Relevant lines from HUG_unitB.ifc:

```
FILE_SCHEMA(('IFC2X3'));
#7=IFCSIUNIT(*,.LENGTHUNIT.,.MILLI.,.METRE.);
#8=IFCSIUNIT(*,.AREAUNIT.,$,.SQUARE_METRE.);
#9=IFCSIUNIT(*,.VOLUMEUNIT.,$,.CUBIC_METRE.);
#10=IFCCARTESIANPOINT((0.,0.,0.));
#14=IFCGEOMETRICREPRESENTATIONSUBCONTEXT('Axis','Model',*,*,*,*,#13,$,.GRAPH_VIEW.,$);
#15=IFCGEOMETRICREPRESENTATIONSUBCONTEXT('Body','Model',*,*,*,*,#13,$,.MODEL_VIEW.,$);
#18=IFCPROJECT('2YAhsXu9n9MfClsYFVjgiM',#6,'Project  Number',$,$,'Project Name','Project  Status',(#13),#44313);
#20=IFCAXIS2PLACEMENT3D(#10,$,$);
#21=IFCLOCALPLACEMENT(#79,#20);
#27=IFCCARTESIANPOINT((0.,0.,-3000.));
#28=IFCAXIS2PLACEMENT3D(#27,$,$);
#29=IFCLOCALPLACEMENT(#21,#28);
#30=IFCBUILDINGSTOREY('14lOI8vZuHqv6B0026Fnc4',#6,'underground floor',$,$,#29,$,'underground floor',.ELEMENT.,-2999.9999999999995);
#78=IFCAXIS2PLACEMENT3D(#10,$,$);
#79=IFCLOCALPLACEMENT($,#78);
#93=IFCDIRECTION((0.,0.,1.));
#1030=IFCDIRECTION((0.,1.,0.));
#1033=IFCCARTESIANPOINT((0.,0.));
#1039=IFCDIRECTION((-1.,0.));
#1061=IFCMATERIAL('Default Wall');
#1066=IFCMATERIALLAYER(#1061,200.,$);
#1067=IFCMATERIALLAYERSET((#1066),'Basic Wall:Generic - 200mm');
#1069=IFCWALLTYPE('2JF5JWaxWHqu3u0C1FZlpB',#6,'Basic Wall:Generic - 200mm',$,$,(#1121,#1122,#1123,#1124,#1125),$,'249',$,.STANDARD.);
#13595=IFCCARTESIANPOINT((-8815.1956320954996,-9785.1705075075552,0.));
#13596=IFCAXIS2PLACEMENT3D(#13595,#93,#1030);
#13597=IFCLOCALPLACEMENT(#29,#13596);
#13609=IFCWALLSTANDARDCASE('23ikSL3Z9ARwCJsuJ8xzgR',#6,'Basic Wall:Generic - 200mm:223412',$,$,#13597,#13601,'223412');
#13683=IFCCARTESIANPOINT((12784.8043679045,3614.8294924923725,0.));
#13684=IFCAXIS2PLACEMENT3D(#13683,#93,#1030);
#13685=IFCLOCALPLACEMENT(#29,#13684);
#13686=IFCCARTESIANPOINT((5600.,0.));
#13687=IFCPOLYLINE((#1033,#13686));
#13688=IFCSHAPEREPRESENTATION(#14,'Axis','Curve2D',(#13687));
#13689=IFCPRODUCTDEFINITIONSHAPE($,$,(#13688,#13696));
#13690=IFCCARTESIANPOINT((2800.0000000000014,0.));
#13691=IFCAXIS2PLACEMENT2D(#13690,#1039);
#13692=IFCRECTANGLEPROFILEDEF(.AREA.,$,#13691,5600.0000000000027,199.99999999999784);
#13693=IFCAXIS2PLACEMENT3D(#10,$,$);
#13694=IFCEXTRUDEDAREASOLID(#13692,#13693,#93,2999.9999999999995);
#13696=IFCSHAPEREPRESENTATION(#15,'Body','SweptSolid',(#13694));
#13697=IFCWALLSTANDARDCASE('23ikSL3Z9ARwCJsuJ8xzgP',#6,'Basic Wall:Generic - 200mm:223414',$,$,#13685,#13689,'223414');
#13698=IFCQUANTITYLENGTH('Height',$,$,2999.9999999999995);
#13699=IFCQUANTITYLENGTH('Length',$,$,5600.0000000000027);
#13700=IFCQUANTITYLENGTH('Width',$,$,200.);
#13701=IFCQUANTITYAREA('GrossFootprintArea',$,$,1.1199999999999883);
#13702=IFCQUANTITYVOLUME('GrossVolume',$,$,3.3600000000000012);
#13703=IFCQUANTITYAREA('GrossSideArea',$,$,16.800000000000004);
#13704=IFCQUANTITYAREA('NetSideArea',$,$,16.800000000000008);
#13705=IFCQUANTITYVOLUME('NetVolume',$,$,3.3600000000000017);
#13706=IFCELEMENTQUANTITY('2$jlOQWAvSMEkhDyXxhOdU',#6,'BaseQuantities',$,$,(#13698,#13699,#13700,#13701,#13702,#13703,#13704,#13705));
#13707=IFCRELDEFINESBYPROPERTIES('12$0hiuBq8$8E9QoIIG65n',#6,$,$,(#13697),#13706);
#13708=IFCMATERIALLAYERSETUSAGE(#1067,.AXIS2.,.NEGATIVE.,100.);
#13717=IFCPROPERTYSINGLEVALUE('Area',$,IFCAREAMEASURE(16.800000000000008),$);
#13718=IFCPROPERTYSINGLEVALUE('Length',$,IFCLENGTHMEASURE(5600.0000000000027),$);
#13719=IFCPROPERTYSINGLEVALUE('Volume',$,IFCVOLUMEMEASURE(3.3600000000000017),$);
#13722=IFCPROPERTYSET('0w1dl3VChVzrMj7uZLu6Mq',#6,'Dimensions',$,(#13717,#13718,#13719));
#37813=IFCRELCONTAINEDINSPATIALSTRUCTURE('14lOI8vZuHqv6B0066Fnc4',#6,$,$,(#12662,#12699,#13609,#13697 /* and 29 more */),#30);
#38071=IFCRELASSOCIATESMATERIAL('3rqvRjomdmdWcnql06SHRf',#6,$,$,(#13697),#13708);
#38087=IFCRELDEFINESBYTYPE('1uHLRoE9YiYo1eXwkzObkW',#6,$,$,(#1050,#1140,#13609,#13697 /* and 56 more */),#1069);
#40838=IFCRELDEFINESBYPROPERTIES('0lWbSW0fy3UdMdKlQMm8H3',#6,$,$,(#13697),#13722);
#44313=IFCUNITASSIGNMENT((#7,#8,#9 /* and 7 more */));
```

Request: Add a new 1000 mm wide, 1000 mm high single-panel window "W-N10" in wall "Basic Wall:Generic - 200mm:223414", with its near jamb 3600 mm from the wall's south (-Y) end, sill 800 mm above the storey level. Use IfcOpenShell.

```python
import numpy as np
import ifcopenshell
import ifcopenshell.api.feature
import ifcopenshell.api.geometry
import ifcopenshell.api.pset
import ifcopenshell.api.root
import ifcopenshell.api.spatial
import ifcopenshell.api.type
import ifcopenshell.geom
import ifcopenshell.util.element
import ifcopenshell.util.placement
import ifcopenshell.util.representation
import ifcopenshell.util.shape
import ifcopenshell.util.unit

model = ifcopenshell.open("HUG_unitB.ifc")
unit_scale = ifcopenshell.util.unit.calculate_unit_scale(model)
area_scale = ifcopenshell.util.unit.calculate_unit_scale(model, "AREAUNIT")
volume_scale = ifcopenshell.util.unit.calculate_unit_scale(model, "VOLUMEUNIT")
settings = ifcopenshell.geom.settings()


def volume(element):
    """Net volume in cubic metres, openings subtracted."""
    shape = ifcopenshell.geom.create_shape(settings, element)
    return ifcopenshell.util.shape.get_volume(shape.geometry)


wall = model.by_guid("23ikSL3Z9ARwCJsuJ8xzgP")
storey = ifcopenshell.util.element.get_container(wall, ifc_class="IfcBuildingStorey")
context = ifcopenshell.util.representation.get_context(model, "Model", "Body", "MODEL_VIEW")
before = volume(wall)

width, height, from_end, sill = 1, 1, 3.6, 0.8  # metres

# The wall runs along its own X axis, and the end named is its -X end.
wall_shape = ifcopenshell.geom.create_shape(settings, wall)
x, y, z = ifcopenshell.util.shape.get_vertices(wall_shape.geometry).T
start = x.min() + from_end
face, thickness = float(y.min()), float(y.max() - y.min())
wall_matrix = ifcopenshell.util.placement.get_local_placement(wall.ObjectPlacement)
level = ifcopenshell.util.placement.get_local_placement(storey.ObjectPlacement)[2, 3]


def in_wall(x, y):
    """Placement at x, y metres in the wall's axes, at sill height."""
    matrix = wall_matrix.copy()
    matrix[:, 3] = wall_matrix @ np.array([x / unit_scale, y / unit_scale, 0.0, 1.0])
    matrix[2, 3] = level + sill / unit_scale
    return matrix


# Opening: a box that overshoots both wall faces by 50 mm.
opening = ifcopenshell.api.root.create_entity(model, ifc_class="IfcOpeningElement")
box = ifcopenshell.api.geometry.add_wall_representation(
    model, context=context, length=width, height=height, thickness=thickness + 0.1
)
ifcopenshell.api.geometry.assign_representation(model, product=opening, representation=box)
ifcopenshell.api.geometry.edit_object_placement(model, product=opening, matrix=in_wall(start, face - 0.05), is_si=False)
ifcopenshell.api.feature.add_feature(model, feature=opening, element=wall)

window = ifcopenshell.api.root.create_entity(model, ifc_class="IfcWindow", name="W-N10")
window.OverallWidth, window.OverallHeight = width / unit_scale, height / unit_scale
body = ifcopenshell.api.geometry.add_window_representation(
    model,
    context=context,
    overall_width=window.OverallWidth,
    overall_height=window.OverallHeight,
    partition_type="SINGLE_PANEL",
)
ifcopenshell.api.geometry.assign_representation(model, product=window, representation=body)
ifcopenshell.api.spatial.assign_container(model, products=[window], relating_structure=storey)
fills = ifcopenshell.api.feature.add_filling(model, opening=opening, element=window)
fills.OwnerHistory = window.OwnerHistory  # required in IFC2X3

# IFC2X3 keeps the operation on the window style.
style = ifcopenshell.api.root.create_entity(model, ifc_class="IfcWindowStyle", name="W-N10")
style.OperationType, style.ConstructionType = "SINGLE_PANEL", "NOTDEFINED"
style.ParameterTakesPrecedence = style.Sizeable = False
ifcopenshell.api.type.assign_type(model, related_objects=[window], relating_type=style)

# Centre the window in the wall's thickness.
ifcopenshell.api.geometry.edit_object_placement(model, product=window, matrix=in_wall(start, face), is_si=False)
window_shape = ifcopenshell.geom.create_shape(settings, window)
depth = ifcopenshell.util.shape.get_vertices(window_shape.geometry)[:, 1]
offset = face + thickness / 2 - (depth.min() + depth.max()) / 2
ifcopenshell.api.geometry.edit_object_placement(model, product=window, matrix=in_wall(start, offset), is_si=False)

after = volume(wall)

# Update the wall's stored quantities.
qto = model.by_id(ifcopenshell.util.element.get_pset(wall, "BaseQuantities", should_inherit=False)["id"])
ifcopenshell.api.pset.edit_qto(model, qto=qto, properties={
    "NetSideArea": after / thickness / area_scale,
    "NetVolume": after / volume_scale,
})
pset = model.by_id(ifcopenshell.util.element.get_pset(wall, "Dimensions", should_inherit=False)["id"])
ifcopenshell.api.pset.edit_pset(model, pset=pset, properties={
    "Area": model.create_entity("IfcAreaMeasure", after / thickness / area_scale),
    "Volume": model.create_entity("IfcVolumeMeasure", after / volume_scale),
})

print(f"wall volume {before:.3f} -> {after:.3f} m3")

model.write("HUG_unitB_edited.ifc")
```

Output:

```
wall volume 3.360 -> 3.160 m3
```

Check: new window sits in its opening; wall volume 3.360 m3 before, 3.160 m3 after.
